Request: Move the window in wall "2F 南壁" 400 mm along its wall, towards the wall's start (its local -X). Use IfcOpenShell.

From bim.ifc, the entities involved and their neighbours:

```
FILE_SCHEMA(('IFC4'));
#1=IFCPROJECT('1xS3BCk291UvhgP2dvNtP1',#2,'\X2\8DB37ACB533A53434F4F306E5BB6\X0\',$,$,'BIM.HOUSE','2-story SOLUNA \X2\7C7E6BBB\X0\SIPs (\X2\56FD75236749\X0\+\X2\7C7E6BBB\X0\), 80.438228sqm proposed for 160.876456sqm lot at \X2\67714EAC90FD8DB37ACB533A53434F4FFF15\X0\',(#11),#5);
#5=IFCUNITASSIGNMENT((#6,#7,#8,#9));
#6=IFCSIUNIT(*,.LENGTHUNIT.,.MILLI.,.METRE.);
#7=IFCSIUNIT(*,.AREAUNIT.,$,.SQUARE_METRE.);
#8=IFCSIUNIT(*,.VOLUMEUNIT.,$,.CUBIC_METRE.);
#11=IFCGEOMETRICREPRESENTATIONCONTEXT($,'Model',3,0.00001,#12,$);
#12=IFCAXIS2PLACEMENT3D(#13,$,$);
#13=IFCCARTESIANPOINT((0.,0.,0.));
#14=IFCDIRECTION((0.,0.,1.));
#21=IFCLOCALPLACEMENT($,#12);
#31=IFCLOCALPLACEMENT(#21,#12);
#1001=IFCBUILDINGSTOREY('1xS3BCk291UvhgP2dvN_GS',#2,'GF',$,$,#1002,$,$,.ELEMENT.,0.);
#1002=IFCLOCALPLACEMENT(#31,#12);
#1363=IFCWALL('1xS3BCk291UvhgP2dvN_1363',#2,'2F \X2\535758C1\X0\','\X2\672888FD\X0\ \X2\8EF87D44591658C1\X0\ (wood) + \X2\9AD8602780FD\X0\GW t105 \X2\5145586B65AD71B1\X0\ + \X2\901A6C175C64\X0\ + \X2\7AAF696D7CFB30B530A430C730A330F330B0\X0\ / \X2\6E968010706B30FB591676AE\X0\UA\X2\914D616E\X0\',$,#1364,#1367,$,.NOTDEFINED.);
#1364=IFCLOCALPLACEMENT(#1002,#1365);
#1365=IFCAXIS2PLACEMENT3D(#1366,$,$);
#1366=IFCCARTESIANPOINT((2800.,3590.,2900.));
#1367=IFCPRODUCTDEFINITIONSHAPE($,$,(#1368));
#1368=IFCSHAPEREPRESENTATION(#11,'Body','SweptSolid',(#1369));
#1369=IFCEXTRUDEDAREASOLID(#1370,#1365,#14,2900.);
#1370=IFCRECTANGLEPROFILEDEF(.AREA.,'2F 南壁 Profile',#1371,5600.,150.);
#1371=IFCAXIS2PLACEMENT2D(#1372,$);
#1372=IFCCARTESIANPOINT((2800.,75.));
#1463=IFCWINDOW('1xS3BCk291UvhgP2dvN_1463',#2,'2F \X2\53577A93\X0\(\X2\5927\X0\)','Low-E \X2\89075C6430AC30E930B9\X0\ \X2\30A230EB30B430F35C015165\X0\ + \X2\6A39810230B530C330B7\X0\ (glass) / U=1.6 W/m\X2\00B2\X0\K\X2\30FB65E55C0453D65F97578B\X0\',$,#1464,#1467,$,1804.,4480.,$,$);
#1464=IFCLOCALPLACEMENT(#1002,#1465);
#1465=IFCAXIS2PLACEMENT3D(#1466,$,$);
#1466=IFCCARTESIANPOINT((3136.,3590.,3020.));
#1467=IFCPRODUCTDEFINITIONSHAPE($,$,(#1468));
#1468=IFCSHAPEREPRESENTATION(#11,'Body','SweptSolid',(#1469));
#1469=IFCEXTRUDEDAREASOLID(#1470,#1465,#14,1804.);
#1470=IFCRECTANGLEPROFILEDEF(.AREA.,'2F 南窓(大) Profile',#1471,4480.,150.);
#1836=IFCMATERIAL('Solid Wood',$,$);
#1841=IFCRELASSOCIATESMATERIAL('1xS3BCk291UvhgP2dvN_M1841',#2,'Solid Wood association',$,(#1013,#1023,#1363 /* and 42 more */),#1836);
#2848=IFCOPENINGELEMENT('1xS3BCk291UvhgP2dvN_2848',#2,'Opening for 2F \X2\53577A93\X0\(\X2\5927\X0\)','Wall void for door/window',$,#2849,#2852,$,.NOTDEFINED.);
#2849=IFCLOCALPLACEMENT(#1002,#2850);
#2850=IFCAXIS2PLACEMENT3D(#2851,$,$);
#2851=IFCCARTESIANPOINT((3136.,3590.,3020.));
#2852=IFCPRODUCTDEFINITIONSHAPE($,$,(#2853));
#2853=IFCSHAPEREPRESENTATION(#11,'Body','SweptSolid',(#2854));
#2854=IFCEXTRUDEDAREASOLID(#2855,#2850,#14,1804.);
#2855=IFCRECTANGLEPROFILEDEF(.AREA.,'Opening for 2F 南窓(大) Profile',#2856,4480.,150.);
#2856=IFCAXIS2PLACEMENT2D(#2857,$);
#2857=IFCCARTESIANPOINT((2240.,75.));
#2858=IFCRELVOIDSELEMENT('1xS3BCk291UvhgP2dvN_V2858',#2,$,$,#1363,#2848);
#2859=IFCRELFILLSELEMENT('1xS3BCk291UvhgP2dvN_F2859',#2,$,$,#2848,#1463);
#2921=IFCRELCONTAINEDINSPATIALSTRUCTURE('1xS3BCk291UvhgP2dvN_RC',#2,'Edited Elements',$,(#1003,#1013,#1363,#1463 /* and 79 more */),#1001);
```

```python
import ifcopenshell
import ifcopenshell.api.geometry
import ifcopenshell.util.placement

model = ifcopenshell.open("bim.ifc")

window = model.by_guid("1xS3BCk291UvhgP2dvN_1463")
opening = window.FillsVoids[0].RelatingOpeningElement
wall = opening.VoidsElements[0].RelatingBuildingElement

wall_matrix = ifcopenshell.util.placement.get_local_placement(wall.ObjectPlacement)
shift = wall_matrix[:3, 0] * -400.0
before = ifcopenshell.util.placement.get_local_placement(window.ObjectPlacement)[:3, 3].copy()

# The window is not placed relative to its opening, so move both.
for product in (opening, window):
    matrix = ifcopenshell.util.placement.get_local_placement(product.ObjectPlacement)
    matrix[:3, 3] += shift
    ifcopenshell.api.geometry.edit_object_placement(model, product=product, matrix=matrix, is_si=False)

after = ifcopenshell.util.placement.get_local_placement(window.ObjectPlacement)[:3, 3]
print("window moved by", (after - before).round(3) + 0.0)

model.write("bim_v2.ifc")
```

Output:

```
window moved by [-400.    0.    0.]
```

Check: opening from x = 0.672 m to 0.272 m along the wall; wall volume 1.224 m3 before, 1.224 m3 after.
